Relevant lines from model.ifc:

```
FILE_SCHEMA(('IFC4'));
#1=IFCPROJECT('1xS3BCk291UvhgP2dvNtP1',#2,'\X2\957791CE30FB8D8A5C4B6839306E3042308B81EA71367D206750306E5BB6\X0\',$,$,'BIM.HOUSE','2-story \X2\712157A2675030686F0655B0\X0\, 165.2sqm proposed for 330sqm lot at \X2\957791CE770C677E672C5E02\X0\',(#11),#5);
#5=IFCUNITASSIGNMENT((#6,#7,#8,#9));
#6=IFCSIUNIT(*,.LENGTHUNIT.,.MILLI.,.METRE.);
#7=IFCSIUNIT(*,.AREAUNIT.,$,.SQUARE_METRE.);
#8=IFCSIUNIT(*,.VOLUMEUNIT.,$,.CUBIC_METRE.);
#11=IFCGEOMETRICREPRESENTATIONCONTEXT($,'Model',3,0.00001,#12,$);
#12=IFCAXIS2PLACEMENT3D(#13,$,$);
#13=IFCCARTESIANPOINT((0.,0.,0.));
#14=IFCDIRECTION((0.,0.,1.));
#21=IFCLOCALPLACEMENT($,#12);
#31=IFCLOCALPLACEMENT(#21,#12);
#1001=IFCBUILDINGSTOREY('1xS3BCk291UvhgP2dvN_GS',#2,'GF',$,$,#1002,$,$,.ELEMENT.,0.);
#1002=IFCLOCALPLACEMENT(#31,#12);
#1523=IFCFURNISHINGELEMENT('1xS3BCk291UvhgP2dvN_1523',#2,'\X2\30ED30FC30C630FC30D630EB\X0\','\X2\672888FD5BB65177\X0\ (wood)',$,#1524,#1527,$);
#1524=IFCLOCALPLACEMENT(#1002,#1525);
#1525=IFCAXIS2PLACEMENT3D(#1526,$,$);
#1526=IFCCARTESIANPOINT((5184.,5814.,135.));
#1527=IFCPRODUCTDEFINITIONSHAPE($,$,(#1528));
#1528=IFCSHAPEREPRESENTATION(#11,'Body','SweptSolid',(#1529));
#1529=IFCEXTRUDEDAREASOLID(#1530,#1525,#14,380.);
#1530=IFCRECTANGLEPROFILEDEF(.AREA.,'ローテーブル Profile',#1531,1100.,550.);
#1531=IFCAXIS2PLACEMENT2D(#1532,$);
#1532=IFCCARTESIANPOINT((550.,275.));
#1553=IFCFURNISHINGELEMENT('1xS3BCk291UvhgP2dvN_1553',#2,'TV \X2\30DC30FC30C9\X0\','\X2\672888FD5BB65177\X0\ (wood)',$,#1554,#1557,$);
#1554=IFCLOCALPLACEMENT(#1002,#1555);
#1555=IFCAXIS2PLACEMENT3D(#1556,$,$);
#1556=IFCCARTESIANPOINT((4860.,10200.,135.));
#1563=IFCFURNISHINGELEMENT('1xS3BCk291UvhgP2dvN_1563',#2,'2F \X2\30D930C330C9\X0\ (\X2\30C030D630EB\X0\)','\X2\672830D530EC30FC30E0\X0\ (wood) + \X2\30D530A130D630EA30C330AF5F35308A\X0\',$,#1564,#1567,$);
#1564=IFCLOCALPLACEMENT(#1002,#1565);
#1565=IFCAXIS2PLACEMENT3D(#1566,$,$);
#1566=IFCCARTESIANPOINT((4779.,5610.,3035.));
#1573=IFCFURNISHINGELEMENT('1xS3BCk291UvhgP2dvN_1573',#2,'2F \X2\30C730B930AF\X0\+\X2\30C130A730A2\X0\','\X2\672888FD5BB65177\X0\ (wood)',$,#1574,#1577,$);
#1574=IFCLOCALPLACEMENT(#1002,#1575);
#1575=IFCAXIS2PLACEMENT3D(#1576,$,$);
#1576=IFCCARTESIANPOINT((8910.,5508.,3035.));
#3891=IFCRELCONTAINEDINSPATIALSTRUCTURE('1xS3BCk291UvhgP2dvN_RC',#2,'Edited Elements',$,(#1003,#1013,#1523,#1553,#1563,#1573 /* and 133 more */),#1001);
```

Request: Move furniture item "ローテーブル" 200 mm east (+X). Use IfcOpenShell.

```python
import ifcopenshell
import ifcopenshell.api.geometry
import ifcopenshell.util.placement

model = ifcopenshell.open("model.ifc")

item = model.by_id(1523)
matrix = ifcopenshell.util.placement.get_local_placement(item.ObjectPlacement)
matrix[0, 3] += 200.0
ifcopenshell.api.geometry.edit_object_placement(model, product=item, matrix=matrix, is_si=False)

print(ifcopenshell.util.placement.get_local_placement(item.ObjectPlacement).round(3) + 0.0)

model.write("model-out.ifc")
```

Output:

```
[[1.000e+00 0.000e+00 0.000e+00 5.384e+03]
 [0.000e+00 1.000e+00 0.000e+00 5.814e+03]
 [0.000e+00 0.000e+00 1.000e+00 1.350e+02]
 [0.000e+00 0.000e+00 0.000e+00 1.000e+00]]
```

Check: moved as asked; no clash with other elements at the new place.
